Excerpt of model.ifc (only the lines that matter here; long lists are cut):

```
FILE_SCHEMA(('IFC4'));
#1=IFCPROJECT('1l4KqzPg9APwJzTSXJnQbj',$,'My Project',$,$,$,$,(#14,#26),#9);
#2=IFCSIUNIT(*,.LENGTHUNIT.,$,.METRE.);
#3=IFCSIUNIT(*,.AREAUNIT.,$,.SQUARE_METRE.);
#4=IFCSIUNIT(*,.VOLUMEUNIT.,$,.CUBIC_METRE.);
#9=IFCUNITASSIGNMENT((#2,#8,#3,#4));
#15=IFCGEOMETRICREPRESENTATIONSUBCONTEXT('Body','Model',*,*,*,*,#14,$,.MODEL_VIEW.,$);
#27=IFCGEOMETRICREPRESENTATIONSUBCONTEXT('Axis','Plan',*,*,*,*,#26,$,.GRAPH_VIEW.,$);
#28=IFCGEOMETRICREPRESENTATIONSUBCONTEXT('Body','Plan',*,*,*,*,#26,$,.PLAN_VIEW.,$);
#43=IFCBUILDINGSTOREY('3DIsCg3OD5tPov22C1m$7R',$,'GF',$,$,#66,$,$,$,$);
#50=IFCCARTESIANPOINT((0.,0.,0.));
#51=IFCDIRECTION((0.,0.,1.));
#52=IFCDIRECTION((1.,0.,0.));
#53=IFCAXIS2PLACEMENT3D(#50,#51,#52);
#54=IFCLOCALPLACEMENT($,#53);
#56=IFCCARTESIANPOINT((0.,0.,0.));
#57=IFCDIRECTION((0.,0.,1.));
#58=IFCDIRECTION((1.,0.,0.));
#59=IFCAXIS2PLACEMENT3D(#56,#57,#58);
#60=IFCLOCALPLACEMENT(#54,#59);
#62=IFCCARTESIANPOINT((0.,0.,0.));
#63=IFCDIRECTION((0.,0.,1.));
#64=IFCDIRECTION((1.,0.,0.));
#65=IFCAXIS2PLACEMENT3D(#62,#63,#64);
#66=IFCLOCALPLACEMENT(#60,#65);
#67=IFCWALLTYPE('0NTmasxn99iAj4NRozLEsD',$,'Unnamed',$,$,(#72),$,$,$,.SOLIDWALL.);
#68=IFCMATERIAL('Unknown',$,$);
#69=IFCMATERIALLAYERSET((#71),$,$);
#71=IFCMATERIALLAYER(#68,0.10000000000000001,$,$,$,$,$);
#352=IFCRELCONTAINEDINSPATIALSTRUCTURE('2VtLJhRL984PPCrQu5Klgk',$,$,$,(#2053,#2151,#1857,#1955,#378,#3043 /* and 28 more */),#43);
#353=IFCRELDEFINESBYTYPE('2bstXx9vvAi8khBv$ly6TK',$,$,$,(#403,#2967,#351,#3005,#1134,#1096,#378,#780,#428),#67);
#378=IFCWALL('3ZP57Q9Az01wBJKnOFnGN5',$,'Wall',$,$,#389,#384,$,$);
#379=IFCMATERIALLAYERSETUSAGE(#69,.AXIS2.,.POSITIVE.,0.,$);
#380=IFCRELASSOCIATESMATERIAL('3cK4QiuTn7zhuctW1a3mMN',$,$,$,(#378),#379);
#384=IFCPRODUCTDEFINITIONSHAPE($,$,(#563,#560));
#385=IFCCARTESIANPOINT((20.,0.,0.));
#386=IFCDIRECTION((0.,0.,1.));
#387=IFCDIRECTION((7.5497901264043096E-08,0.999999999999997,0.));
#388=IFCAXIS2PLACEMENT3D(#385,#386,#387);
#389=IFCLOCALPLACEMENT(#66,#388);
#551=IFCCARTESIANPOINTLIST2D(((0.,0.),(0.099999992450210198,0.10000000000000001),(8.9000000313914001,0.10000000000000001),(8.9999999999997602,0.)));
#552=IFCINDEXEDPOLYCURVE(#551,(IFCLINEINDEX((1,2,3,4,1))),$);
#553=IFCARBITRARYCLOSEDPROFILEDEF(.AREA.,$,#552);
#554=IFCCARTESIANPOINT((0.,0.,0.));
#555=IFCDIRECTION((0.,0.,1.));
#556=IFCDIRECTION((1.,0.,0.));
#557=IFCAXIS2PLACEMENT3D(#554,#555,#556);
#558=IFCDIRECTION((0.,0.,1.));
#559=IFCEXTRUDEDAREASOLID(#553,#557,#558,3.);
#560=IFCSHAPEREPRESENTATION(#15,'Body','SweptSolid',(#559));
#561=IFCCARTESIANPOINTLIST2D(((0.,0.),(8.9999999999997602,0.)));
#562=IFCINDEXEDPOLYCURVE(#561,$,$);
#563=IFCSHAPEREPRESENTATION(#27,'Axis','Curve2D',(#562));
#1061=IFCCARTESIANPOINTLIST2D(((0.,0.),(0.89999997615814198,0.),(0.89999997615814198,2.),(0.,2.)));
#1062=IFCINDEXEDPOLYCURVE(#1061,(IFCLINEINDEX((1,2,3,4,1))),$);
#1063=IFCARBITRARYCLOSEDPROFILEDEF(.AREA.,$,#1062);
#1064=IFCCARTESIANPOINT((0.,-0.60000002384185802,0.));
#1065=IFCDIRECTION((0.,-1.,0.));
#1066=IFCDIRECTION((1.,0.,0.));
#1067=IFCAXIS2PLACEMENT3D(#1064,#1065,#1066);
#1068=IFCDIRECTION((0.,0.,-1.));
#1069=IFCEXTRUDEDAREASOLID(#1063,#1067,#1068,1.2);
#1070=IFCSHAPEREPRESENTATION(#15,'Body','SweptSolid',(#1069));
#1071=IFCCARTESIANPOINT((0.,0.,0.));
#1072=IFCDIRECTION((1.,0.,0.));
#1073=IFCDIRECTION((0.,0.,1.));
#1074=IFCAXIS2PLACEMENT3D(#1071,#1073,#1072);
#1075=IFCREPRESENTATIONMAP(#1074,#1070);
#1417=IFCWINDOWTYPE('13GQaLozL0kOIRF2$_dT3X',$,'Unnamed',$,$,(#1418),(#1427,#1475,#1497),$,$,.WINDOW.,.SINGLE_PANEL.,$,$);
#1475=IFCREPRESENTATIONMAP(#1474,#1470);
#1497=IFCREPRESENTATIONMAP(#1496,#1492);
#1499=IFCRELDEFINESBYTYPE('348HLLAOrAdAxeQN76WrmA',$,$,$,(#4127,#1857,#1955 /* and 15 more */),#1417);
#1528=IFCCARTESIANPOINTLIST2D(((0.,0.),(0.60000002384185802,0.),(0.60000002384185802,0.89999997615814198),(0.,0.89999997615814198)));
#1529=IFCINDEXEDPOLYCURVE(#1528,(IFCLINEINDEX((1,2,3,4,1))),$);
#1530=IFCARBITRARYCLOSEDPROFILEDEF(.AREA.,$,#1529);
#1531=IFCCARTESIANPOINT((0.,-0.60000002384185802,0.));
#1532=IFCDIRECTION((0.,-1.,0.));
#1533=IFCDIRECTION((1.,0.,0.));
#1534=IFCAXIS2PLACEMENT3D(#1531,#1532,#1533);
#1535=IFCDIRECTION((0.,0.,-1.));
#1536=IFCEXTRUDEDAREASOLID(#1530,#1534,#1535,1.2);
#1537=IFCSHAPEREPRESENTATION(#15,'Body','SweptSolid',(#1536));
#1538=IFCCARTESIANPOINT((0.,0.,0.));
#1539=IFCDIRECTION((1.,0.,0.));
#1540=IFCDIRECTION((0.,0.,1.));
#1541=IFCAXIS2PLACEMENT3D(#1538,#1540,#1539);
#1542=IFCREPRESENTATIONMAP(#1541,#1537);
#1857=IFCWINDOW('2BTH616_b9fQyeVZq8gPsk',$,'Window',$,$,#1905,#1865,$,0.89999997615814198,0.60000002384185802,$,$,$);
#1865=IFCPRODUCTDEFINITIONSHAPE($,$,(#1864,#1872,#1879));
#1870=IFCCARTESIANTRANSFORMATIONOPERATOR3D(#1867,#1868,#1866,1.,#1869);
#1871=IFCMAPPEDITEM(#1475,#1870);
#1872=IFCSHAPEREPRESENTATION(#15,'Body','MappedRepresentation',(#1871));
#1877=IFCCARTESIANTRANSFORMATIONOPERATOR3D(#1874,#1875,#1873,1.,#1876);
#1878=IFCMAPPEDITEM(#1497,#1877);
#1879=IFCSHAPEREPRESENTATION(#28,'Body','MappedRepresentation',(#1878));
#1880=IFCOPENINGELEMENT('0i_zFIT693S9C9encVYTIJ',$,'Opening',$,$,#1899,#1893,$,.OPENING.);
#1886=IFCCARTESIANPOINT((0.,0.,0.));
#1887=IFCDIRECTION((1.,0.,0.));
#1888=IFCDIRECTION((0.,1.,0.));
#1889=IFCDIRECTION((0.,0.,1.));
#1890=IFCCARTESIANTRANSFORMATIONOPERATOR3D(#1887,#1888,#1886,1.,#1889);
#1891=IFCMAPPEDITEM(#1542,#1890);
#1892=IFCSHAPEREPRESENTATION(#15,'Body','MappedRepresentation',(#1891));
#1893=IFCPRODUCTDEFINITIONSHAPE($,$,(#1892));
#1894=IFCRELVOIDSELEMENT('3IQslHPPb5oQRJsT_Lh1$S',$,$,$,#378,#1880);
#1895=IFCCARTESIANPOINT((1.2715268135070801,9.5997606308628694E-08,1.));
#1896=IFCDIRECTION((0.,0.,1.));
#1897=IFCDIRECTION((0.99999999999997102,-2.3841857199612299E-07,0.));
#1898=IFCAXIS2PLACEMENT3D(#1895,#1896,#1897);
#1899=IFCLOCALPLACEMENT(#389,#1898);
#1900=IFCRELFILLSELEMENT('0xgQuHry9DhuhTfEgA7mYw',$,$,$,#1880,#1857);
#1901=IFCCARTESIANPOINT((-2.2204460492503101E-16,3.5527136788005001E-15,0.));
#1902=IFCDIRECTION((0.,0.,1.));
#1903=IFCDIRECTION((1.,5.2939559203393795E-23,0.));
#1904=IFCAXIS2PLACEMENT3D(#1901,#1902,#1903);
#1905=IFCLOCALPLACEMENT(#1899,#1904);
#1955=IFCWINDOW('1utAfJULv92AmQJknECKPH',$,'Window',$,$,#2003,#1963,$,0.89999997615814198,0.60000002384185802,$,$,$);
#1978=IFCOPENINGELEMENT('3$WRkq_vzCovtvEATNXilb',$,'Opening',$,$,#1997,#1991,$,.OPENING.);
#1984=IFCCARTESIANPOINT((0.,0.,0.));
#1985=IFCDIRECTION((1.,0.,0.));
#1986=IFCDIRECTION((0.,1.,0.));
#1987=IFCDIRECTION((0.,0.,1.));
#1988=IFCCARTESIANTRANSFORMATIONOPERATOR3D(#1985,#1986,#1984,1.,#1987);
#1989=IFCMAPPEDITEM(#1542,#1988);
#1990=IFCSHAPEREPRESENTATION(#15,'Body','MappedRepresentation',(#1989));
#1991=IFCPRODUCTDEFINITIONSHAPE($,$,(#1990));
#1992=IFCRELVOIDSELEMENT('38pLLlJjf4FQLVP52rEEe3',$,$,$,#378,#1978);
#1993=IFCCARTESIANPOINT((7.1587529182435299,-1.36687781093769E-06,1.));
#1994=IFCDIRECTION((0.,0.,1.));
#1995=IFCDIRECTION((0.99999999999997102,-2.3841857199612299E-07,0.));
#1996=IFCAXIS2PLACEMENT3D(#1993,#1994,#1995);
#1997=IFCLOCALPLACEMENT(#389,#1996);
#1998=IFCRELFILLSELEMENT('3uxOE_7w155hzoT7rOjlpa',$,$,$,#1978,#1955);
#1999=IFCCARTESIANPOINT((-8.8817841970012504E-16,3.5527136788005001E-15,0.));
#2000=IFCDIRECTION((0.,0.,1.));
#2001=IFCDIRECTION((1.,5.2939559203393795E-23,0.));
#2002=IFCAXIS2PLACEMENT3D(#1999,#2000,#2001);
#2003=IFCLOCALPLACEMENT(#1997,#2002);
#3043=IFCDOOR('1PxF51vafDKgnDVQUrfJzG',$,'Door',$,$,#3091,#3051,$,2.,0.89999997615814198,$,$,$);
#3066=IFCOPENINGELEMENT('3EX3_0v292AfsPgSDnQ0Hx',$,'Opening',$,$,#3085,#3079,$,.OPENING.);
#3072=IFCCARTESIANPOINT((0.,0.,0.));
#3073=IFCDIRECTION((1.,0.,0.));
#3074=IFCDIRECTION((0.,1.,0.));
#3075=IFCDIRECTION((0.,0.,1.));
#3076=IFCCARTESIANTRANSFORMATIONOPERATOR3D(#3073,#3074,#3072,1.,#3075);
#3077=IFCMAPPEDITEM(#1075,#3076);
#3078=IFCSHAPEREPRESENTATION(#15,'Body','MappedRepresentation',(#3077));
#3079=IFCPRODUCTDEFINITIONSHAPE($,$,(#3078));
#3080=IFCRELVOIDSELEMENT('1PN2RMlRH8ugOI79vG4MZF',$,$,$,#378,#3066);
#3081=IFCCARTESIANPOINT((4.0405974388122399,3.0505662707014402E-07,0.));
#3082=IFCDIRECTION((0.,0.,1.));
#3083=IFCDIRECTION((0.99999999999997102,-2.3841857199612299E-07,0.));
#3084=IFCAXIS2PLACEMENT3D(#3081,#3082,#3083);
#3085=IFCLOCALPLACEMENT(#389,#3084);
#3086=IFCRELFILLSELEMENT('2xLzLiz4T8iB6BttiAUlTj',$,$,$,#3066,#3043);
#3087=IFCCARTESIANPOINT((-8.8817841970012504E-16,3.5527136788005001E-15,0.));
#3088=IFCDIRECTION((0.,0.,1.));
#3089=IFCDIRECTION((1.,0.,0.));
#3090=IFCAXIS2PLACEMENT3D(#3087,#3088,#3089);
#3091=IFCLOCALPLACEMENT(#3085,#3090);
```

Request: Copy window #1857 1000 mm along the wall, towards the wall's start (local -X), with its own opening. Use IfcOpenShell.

```python
import ifcopenshell
import ifcopenshell.api.feature
import ifcopenshell.api.geometry
import ifcopenshell.api.root
import ifcopenshell.geom
import ifcopenshell.util.element
import ifcopenshell.util.placement
import ifcopenshell.util.shape
import ifcopenshell.util.unit

model = ifcopenshell.open("model.ifc")
unit_scale = ifcopenshell.util.unit.calculate_unit_scale(model)
settings = ifcopenshell.geom.settings()


def volume(element):
    """Net volume in cubic metres, openings subtracted."""
    shape = ifcopenshell.geom.create_shape(settings, element)
    return ifcopenshell.util.shape.get_volume(shape.geometry)


window = model.by_id(1857)
opening = window.FillsVoids[0].RelatingOpeningElement
wall = opening.VoidsElements[0].RelatingBuildingElement
before = volume(wall)
shift = ifcopenshell.util.placement.get_local_placement(wall.ObjectPlacement)[:3, 0] * -1 / unit_scale

# copy_class copies the void relationship, type, container and properties, but no geometry.
new_opening = ifcopenshell.api.root.copy_class(model, product=opening)
new_opening.Representation = ifcopenshell.util.element.copy_deep(
    model, opening.Representation, exclude=["IfcGeometricRepresentationContext", "IfcRepresentationMap"]
)
new_window = ifcopenshell.api.root.copy_class(model, product=window)
new_window.Representation = ifcopenshell.util.element.copy_deep(
    model, window.Representation, exclude=["IfcGeometricRepresentationContext", "IfcRepresentationMap"]
)
ifcopenshell.api.feature.add_filling(model, opening=new_opening, element=new_window)

for old, new in ((opening, new_opening), (window, new_window)):
    matrix = ifcopenshell.util.placement.get_local_placement(old.ObjectPlacement)
    matrix[:3, 3] += shift
    ifcopenshell.api.geometry.edit_object_placement(model, product=new, matrix=matrix, is_si=False)

after = volume(wall)

print(f"wall volume {before:.3f} -> {after:.3f} m3")

model.write("model_v2.ifc")
```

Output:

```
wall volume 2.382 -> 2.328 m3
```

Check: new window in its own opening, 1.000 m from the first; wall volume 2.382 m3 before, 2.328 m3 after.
